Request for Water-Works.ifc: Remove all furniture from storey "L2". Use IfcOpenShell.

First a look at what the model holds.

```python
import ifcopenshell
import ifcopenshell.util.element

model = ifcopenshell.open("Water-Works.ifc")
print(model.schema)
storey = next(s for s in model.by_type("IfcBuildingStorey") if s.Name == "L2")
furniture = [e for e in ifcopenshell.util.element.get_decomposition(storey) if e.is_a("IfcFurnishingElement")]
seen = {}
for e in furniture:
    element_type = ifcopenshell.util.element.get_type(e)
    name = element_type.Name if element_type not in (None, e) else None
    seen[name] = seen.get(name, 0) + 1
for name, count in sorted(seen.items(), key=str):
    print(count, "x", name)
```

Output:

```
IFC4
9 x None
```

```python
import ifcopenshell
import ifcopenshell.api.root
import ifcopenshell.util.element

model = ifcopenshell.open("Water-Works.ifc")

storey = next(s for s in model.by_type("IfcBuildingStorey") if s.Name == "L2")
furniture = [e for e in ifcopenshell.util.element.get_decomposition(storey) if e.is_a("IfcFurnishingElement")]

for e in furniture:
    ifcopenshell.api.root.remove_product(model, product=e)
print(len(furniture), "removed")

model.write("Water-Works_updated.ifc")
```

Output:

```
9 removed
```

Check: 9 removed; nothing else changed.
